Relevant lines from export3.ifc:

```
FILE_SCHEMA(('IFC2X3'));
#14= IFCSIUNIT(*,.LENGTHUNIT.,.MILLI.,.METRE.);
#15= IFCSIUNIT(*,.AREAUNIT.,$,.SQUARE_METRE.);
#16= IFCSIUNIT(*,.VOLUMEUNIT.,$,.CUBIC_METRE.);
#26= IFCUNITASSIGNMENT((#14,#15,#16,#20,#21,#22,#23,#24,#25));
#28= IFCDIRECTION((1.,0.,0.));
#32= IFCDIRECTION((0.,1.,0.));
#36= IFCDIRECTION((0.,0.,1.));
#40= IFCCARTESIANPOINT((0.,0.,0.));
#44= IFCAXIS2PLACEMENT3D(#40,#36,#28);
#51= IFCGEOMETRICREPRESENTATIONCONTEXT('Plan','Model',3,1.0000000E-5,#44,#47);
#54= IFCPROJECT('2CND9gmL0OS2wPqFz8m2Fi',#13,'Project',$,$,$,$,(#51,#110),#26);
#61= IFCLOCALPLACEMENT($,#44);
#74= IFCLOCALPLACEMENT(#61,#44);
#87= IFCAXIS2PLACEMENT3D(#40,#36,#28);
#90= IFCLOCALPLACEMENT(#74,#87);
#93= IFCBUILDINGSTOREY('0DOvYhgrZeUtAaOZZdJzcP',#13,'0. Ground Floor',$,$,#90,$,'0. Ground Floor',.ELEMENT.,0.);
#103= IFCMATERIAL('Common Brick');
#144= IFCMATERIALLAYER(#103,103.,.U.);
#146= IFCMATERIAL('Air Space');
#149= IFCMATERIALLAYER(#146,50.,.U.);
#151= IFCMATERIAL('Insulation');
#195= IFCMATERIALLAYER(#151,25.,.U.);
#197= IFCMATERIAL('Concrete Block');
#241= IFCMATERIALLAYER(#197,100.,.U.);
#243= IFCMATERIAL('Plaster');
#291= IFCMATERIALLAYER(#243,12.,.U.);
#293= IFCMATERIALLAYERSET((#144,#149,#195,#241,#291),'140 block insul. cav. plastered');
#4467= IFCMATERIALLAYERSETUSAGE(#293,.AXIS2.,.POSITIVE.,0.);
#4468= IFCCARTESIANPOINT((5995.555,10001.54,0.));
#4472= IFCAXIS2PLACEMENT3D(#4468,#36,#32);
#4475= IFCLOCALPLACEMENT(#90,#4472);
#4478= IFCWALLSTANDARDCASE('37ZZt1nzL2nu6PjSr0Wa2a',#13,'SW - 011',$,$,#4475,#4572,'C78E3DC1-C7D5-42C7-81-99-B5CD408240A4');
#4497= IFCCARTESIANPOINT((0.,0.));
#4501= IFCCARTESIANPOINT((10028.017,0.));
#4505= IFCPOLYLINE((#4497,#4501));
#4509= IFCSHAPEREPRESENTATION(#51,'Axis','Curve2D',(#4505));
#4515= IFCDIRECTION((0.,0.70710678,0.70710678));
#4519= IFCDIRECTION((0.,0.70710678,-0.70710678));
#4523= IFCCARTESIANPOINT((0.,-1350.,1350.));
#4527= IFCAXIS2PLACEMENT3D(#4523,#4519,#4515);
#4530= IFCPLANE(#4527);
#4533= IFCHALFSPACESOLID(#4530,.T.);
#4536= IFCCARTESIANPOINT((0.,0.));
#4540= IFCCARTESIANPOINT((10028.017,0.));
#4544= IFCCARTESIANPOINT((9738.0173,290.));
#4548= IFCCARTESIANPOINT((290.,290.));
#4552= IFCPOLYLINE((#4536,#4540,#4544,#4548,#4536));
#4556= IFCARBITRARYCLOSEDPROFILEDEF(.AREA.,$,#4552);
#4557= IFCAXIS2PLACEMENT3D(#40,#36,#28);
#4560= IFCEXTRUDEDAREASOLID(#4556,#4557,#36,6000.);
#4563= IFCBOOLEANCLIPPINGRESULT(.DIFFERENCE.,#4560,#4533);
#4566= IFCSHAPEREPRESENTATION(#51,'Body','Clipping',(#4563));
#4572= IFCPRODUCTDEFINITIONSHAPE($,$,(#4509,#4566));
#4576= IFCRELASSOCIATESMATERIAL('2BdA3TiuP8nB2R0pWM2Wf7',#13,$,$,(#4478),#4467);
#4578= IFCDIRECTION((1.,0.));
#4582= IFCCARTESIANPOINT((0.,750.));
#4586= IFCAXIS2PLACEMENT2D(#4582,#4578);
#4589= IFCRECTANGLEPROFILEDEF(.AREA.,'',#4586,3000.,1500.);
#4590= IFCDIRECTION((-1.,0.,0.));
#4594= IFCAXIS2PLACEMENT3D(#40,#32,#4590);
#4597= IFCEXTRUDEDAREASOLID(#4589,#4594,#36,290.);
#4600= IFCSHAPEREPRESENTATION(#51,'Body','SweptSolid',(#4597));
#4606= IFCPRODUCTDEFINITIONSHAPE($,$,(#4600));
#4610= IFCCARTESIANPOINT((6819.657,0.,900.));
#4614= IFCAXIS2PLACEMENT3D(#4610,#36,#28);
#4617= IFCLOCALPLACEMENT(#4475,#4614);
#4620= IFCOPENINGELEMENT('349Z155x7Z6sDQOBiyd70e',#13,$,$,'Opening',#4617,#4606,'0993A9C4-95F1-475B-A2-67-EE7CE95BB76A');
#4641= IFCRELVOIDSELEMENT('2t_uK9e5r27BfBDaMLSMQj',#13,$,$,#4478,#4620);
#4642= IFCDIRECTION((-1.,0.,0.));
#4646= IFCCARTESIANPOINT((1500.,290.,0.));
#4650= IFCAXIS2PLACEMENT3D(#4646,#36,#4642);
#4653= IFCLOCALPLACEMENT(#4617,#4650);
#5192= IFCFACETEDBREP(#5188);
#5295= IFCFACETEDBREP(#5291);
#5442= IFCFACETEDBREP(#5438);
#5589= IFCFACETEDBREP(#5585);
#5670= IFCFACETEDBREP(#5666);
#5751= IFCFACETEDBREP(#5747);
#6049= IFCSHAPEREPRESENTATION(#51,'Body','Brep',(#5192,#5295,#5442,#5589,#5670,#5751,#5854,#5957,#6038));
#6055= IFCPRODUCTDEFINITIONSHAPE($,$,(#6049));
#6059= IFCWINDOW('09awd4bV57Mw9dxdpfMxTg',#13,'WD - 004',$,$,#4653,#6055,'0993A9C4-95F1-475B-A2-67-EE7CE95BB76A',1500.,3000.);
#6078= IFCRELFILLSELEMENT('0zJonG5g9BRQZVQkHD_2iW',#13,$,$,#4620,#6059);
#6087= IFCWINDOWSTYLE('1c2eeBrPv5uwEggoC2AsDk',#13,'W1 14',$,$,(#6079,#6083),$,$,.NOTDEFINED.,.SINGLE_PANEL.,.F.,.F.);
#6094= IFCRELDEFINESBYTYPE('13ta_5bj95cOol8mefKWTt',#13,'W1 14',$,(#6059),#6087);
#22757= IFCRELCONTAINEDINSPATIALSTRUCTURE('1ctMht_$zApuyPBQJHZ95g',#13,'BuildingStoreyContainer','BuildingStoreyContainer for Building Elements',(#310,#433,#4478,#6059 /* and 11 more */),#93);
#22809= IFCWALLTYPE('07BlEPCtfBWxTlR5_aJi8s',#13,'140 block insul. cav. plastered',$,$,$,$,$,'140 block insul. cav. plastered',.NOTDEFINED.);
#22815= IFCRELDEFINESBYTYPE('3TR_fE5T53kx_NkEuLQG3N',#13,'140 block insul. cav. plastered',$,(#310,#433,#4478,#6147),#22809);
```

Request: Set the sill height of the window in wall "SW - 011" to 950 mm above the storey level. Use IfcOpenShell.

```python
import numpy as np
import ifcopenshell
import ifcopenshell.api.geometry
import ifcopenshell.geom
import ifcopenshell.util.element
import ifcopenshell.util.placement
import ifcopenshell.util.shape
import ifcopenshell.util.unit

model = ifcopenshell.open("export3.ifc")
unit_scale = ifcopenshell.util.unit.calculate_unit_scale(model)

window = model.by_guid("09awd4bV57Mw9dxdpfMxTg")
opening = window.FillsVoids[0].RelatingOpeningElement
storey = ifcopenshell.util.element.get_container(window, ifc_class="IfcBuildingStorey")
level = ifcopenshell.util.placement.get_local_placement(storey.ObjectPlacement)[2, 3]

# The opening's origin need not be at the sill, so measure its lowest point.
shape = ifcopenshell.geom.create_shape(ifcopenshell.geom.settings(), opening)
bottom = ifcopenshell.util.shape.get_shape_bottom_elevation(shape, shape.geometry) / unit_scale
dz = level + 0.95 / unit_scale - bottom

shift = np.array([0.0, 0.0, dz])
# The window is placed relative to its opening, so it follows when the opening moves.
matrix = ifcopenshell.util.placement.get_local_placement(opening.ObjectPlacement)
matrix[:3, 3] += shift
ifcopenshell.api.geometry.edit_object_placement(
    model, product=opening, matrix=matrix, is_si=False, should_transform_children=True
)

print(f"moved by {dz * unit_scale:+.3f} m")

model.write("export3_rev.ifc")
```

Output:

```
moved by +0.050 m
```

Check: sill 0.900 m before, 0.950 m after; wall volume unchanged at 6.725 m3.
